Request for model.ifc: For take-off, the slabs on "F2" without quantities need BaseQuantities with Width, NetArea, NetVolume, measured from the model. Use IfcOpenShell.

First a look at what the model holds.

```python
import ifcopenshell
import ifcopenshell.util.element
import ifcopenshell.util.unit

model = ifcopenshell.open("model.ifc")
print(model.schema)
for unit_type in ("LENGTHUNIT", "AREAUNIT", "VOLUMEUNIT"):
    print(unit_type, ifcopenshell.util.unit.calculate_unit_scale(model, unit_type))
storey = next(s for s in model.by_type("IfcBuildingStorey") if s.Name == "F2")
slabs = [e for e in ifcopenshell.util.element.get_decomposition(storey) if e.is_a("IfcSlab")]
for e in sorted(slabs, key=lambda e: e.id()):
    print(e.id(), e.is_a(), e.Name, list(ifcopenshell.util.element.get_psets(e, qtos_only=True)), sep=" | ")
```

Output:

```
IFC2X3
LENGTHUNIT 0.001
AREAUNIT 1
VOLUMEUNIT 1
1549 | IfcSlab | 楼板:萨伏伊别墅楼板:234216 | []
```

```python
import ifcopenshell
import ifcopenshell.api.pset
import ifcopenshell.geom
import ifcopenshell.util.element
import ifcopenshell.util.shape
import ifcopenshell.util.unit

model = ifcopenshell.open("model.ifc")
unit_scale = ifcopenshell.util.unit.calculate_unit_scale(model)
area_scale = ifcopenshell.util.unit.calculate_unit_scale(model, "AREAUNIT")
volume_scale = ifcopenshell.util.unit.calculate_unit_scale(model, "VOLUMEUNIT")
settings = ifcopenshell.geom.settings()

storey = next(s for s in model.by_type("IfcBuildingStorey") if s.Name == "F2")
slabs = [e for e in ifcopenshell.util.element.get_decomposition(storey) if e.is_a("IfcSlab")]

for e in sorted(slabs, key=lambda e: e.id()):
    if ifcopenshell.util.element.get_psets(e, qtos_only=True, should_inherit=False):
        continue
    # Geometry comes back in metres, in the element's own axes.
    shape = ifcopenshell.geom.create_shape(settings, e)
    values = {
        "Width": ifcopenshell.util.shape.get_z(shape.geometry) / unit_scale,
        "NetArea": ifcopenshell.util.shape.get_footprint_area(shape.geometry) / area_scale,
        "NetVolume": ifcopenshell.util.shape.get_volume(shape.geometry) / volume_scale,
    }
    qto = ifcopenshell.api.pset.add_qto(model, product=e, name="BaseQuantities")
    ifcopenshell.api.pset.edit_qto(model, qto=qto, properties=values)
    print(e.id(), {k: round(v, 3) for k, v in values.items()})

model.write("model-out.ifc")
```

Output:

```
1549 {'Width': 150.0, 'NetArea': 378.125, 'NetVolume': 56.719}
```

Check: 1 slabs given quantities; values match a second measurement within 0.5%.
